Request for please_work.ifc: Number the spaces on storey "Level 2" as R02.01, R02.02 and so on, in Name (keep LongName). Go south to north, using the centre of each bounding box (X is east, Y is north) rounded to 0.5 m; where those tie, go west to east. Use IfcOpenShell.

First a look at what the model holds.

```python
import ifcopenshell
import ifcopenshell.util.element
import ifcopenshell.util.placement

model = ifcopenshell.open("please_work.ifc")
print(model.schema)
storey = next(s for s in model.by_type("IfcBuildingStorey") if s.Name == "Level 2")
spaces = [e for e in ifcopenshell.util.element.get_decomposition(storey) if e.is_a("IfcSpace")]
for e in sorted(spaces, key=lambda e: e.id()):
    origin = ifcopenshell.util.placement.get_local_placement(e.ObjectPlacement)[:3, 3]
    print(e.id(), e.Name, e.LongName, origin.round(2) + 0.0, sep=" | ")
```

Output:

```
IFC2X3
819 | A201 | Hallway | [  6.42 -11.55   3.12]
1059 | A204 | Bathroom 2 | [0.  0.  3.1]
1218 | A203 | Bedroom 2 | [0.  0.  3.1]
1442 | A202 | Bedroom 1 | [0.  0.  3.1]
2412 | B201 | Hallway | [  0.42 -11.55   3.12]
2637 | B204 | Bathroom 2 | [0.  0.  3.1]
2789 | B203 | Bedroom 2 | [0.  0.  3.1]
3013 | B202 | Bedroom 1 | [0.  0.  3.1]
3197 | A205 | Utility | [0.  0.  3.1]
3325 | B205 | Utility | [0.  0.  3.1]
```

```python
import ifcopenshell
import ifcopenshell.geom
import ifcopenshell.util.element
import ifcopenshell.util.shape

model = ifcopenshell.open("please_work.ifc")
settings = ifcopenshell.geom.settings()
settings.set("use-world-coords", True)


def centre(element):
    shape = ifcopenshell.geom.create_shape(settings, element)
    return ifcopenshell.util.shape.get_bbox_centroid(shape.geometry)


storey = next(s for s in model.by_type("IfcBuildingStorey") if s.Name == "Level 2")
spaces = [e for e in ifcopenshell.util.element.get_decomposition(storey) if e.is_a("IfcSpace")]

# Insertion points can sit at a corner or the storey origin, so sort by the geometry (in metres).
centres = {e: centre(e) for e in spaces}
spaces.sort(key=lambda e: (round(centres[e][1] / 0.5), centres[e][0]))

for i, e in enumerate(spaces, start=1):
    number = f"R02.{i:02d}"
    e.Name = number
    print(e.id(), number)

model.write("please_work_edited.ifc")
```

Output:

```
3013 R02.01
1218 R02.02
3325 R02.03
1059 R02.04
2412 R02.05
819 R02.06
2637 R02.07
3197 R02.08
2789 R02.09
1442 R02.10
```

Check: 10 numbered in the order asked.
